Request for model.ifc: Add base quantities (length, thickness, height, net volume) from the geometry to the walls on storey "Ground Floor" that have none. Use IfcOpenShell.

First a look at what the model holds.

```python
import ifcopenshell
import ifcopenshell.util.element
import ifcopenshell.util.unit

model = ifcopenshell.open("model.ifc")
print(model.schema)
for unit_type in ("LENGTHUNIT", "AREAUNIT", "VOLUMEUNIT"):
    print(unit_type, ifcopenshell.util.unit.calculate_unit_scale(model, unit_type))
storey = next(s for s in model.by_type("IfcBuildingStorey") if s.Name == "Ground Floor")
walls = [e for e in ifcopenshell.util.element.get_decomposition(storey) if e.is_a("IfcWall")]
for e in sorted(walls, key=lambda e: e.id()):
    print(e.id(), e.is_a(), e.Name, list(ifcopenshell.util.element.get_psets(e, qtos_only=True)), sep=" | ")
```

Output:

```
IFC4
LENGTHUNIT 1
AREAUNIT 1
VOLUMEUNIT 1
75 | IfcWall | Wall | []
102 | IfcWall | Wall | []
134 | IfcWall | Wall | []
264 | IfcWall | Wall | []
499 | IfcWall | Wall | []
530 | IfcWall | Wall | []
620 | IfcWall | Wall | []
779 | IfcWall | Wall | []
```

```python
import ifcopenshell
import ifcopenshell.api.pset
import ifcopenshell.geom
import ifcopenshell.util.element
import ifcopenshell.util.shape
import ifcopenshell.util.unit

model = ifcopenshell.open("model.ifc")
unit_scale = ifcopenshell.util.unit.calculate_unit_scale(model)
volume_scale = ifcopenshell.util.unit.calculate_unit_scale(model, "VOLUMEUNIT")
settings = ifcopenshell.geom.settings()

storey = next(s for s in model.by_type("IfcBuildingStorey") if s.Name == "Ground Floor")
walls = [e for e in ifcopenshell.util.element.get_decomposition(storey) if e.is_a("IfcWall")]

for e in sorted(walls, key=lambda e: e.id()):
    if ifcopenshell.util.element.get_psets(e, qtos_only=True, should_inherit=False):
        continue
    # Geometry comes back in metres, in the element's own axes.
    shape = ifcopenshell.geom.create_shape(settings, e)
    values = {
        "Length": ifcopenshell.util.shape.get_x(shape.geometry) / unit_scale,
        "Width": ifcopenshell.util.shape.get_y(shape.geometry) / unit_scale,
        "Height": ifcopenshell.util.shape.get_z(shape.geometry) / unit_scale,
        "NetVolume": ifcopenshell.util.shape.get_volume(shape.geometry) / volume_scale,
    }
    qto = ifcopenshell.api.pset.add_qto(model, product=e, name="Qto_WallBaseQuantities")
    ifcopenshell.api.pset.edit_qto(model, qto=qto, properties=values)
    print(e.id(), {k: round(v, 3) for k, v in values.items()})

model.write("model_v2.ifc")
```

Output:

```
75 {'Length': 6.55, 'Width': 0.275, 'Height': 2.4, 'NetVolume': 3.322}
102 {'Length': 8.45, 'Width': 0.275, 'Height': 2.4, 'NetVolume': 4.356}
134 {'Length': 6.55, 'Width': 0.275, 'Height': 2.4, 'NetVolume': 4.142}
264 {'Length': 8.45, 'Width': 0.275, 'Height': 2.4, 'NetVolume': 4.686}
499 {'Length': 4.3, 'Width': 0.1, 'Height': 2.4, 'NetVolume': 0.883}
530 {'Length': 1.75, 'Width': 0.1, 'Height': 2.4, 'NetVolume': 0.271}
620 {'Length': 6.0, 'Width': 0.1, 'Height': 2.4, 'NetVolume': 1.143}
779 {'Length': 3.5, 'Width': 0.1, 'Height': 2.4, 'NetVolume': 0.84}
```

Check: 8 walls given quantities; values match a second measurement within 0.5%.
